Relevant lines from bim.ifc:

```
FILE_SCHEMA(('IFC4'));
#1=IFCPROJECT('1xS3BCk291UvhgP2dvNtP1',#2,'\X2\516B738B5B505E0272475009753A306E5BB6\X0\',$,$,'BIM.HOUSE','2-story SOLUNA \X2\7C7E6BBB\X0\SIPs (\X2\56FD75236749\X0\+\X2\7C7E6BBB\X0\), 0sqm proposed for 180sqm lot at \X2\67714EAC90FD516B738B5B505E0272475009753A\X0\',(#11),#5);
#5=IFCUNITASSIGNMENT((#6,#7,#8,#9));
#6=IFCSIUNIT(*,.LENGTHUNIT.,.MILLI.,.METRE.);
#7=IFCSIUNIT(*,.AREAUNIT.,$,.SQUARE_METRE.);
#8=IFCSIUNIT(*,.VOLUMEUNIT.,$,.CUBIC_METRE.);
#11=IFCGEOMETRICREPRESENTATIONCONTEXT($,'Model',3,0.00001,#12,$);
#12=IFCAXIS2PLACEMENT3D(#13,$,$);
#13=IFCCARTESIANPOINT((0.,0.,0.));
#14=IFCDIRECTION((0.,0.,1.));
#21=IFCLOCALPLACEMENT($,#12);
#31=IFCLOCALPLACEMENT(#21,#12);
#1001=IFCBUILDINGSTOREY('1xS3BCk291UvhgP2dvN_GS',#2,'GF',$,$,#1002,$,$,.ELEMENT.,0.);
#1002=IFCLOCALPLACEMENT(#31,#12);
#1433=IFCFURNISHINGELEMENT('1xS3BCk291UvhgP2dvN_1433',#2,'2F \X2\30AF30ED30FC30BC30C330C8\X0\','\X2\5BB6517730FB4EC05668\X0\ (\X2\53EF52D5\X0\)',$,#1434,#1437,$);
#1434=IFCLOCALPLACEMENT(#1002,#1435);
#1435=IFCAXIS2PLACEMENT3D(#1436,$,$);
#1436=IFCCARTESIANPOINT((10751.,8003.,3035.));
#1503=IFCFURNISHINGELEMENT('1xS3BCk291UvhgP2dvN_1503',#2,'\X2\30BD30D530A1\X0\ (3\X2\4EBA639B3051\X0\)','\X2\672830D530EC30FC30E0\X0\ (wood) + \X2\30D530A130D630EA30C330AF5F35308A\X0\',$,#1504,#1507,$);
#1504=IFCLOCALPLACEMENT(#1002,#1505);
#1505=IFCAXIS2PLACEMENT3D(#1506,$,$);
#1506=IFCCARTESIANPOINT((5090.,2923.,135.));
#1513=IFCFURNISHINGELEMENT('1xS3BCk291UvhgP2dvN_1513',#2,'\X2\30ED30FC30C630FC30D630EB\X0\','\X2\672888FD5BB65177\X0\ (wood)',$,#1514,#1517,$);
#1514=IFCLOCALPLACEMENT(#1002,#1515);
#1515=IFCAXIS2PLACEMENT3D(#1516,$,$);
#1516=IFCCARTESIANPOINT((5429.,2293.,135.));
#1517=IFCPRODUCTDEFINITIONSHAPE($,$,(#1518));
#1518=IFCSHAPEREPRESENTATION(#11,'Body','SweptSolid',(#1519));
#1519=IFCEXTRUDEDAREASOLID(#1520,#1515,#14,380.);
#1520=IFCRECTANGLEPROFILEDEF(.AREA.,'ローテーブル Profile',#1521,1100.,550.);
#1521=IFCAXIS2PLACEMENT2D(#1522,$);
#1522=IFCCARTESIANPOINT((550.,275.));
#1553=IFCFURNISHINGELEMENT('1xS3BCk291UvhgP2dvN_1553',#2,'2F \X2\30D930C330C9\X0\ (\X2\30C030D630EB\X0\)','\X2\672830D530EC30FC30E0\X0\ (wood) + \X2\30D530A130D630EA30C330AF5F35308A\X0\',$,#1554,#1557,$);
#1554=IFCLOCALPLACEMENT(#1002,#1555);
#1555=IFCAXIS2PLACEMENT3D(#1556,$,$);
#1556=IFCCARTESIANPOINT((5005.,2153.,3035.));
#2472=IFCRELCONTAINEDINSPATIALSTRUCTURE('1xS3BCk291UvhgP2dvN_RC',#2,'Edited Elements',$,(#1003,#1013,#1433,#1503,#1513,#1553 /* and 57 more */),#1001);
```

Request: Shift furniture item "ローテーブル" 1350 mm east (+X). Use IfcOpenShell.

```python
import ifcopenshell
import ifcopenshell.api.geometry
import ifcopenshell.util.placement
import ifcopenshell.util.unit

model = ifcopenshell.open("bim.ifc")
unit_scale = ifcopenshell.util.unit.calculate_unit_scale(model)

item = model.by_guid("1xS3BCk291UvhgP2dvN_1513")
matrix = ifcopenshell.util.placement.get_local_placement(item.ObjectPlacement)
matrix[0, 3] += 1.35 / unit_scale
ifcopenshell.api.geometry.edit_object_placement(model, product=item, matrix=matrix, is_si=False)

print(ifcopenshell.util.placement.get_local_placement(item.ObjectPlacement).round(3) + 0.0)

model.write("bim_edited.ifc")
```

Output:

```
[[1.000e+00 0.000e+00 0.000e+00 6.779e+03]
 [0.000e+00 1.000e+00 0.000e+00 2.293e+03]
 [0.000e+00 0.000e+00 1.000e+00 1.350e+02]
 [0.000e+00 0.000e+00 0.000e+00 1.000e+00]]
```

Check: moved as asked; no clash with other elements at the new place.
